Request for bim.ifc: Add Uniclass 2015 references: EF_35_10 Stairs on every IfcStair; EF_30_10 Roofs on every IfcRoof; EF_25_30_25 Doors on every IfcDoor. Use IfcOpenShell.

First a look at what the model holds.

```python
import ifcopenshell

model = ifcopenshell.open("bim.ifc")
print(model.schema)
print("classifications:", [c.Name for c in model.by_type("IfcClassification")])
for ifc_class in ("IfcDoor", "IfcRoof", "IfcStair", "IfcWall", "IfcWindow"):
    print(ifc_class, len(model.by_type(ifc_class)))
```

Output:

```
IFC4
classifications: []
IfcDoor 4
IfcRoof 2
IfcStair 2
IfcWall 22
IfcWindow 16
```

```python
import ifcopenshell
import ifcopenshell.api.classification

model = ifcopenshell.open("bim.ifc")

system = ifcopenshell.api.classification.add_classification(model, classification="Uniclass 2015")

codes = {
    "IfcStair": ("EF_35_10", "Stairs"),
    "IfcRoof": ("EF_30_10", "Roofs"),
    "IfcDoor": ("EF_25_30_25", "Doors"),
}
for ifc_class, (code, name) in codes.items():
    products = model.by_type(ifc_class)
    ifcopenshell.api.classification.add_reference(
        model, products=products, classification=system, identification=code, name=name
    )
    print(code, len(products))

model.write("bim_rev.ifc")
```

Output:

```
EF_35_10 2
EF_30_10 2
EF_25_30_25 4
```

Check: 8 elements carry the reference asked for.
